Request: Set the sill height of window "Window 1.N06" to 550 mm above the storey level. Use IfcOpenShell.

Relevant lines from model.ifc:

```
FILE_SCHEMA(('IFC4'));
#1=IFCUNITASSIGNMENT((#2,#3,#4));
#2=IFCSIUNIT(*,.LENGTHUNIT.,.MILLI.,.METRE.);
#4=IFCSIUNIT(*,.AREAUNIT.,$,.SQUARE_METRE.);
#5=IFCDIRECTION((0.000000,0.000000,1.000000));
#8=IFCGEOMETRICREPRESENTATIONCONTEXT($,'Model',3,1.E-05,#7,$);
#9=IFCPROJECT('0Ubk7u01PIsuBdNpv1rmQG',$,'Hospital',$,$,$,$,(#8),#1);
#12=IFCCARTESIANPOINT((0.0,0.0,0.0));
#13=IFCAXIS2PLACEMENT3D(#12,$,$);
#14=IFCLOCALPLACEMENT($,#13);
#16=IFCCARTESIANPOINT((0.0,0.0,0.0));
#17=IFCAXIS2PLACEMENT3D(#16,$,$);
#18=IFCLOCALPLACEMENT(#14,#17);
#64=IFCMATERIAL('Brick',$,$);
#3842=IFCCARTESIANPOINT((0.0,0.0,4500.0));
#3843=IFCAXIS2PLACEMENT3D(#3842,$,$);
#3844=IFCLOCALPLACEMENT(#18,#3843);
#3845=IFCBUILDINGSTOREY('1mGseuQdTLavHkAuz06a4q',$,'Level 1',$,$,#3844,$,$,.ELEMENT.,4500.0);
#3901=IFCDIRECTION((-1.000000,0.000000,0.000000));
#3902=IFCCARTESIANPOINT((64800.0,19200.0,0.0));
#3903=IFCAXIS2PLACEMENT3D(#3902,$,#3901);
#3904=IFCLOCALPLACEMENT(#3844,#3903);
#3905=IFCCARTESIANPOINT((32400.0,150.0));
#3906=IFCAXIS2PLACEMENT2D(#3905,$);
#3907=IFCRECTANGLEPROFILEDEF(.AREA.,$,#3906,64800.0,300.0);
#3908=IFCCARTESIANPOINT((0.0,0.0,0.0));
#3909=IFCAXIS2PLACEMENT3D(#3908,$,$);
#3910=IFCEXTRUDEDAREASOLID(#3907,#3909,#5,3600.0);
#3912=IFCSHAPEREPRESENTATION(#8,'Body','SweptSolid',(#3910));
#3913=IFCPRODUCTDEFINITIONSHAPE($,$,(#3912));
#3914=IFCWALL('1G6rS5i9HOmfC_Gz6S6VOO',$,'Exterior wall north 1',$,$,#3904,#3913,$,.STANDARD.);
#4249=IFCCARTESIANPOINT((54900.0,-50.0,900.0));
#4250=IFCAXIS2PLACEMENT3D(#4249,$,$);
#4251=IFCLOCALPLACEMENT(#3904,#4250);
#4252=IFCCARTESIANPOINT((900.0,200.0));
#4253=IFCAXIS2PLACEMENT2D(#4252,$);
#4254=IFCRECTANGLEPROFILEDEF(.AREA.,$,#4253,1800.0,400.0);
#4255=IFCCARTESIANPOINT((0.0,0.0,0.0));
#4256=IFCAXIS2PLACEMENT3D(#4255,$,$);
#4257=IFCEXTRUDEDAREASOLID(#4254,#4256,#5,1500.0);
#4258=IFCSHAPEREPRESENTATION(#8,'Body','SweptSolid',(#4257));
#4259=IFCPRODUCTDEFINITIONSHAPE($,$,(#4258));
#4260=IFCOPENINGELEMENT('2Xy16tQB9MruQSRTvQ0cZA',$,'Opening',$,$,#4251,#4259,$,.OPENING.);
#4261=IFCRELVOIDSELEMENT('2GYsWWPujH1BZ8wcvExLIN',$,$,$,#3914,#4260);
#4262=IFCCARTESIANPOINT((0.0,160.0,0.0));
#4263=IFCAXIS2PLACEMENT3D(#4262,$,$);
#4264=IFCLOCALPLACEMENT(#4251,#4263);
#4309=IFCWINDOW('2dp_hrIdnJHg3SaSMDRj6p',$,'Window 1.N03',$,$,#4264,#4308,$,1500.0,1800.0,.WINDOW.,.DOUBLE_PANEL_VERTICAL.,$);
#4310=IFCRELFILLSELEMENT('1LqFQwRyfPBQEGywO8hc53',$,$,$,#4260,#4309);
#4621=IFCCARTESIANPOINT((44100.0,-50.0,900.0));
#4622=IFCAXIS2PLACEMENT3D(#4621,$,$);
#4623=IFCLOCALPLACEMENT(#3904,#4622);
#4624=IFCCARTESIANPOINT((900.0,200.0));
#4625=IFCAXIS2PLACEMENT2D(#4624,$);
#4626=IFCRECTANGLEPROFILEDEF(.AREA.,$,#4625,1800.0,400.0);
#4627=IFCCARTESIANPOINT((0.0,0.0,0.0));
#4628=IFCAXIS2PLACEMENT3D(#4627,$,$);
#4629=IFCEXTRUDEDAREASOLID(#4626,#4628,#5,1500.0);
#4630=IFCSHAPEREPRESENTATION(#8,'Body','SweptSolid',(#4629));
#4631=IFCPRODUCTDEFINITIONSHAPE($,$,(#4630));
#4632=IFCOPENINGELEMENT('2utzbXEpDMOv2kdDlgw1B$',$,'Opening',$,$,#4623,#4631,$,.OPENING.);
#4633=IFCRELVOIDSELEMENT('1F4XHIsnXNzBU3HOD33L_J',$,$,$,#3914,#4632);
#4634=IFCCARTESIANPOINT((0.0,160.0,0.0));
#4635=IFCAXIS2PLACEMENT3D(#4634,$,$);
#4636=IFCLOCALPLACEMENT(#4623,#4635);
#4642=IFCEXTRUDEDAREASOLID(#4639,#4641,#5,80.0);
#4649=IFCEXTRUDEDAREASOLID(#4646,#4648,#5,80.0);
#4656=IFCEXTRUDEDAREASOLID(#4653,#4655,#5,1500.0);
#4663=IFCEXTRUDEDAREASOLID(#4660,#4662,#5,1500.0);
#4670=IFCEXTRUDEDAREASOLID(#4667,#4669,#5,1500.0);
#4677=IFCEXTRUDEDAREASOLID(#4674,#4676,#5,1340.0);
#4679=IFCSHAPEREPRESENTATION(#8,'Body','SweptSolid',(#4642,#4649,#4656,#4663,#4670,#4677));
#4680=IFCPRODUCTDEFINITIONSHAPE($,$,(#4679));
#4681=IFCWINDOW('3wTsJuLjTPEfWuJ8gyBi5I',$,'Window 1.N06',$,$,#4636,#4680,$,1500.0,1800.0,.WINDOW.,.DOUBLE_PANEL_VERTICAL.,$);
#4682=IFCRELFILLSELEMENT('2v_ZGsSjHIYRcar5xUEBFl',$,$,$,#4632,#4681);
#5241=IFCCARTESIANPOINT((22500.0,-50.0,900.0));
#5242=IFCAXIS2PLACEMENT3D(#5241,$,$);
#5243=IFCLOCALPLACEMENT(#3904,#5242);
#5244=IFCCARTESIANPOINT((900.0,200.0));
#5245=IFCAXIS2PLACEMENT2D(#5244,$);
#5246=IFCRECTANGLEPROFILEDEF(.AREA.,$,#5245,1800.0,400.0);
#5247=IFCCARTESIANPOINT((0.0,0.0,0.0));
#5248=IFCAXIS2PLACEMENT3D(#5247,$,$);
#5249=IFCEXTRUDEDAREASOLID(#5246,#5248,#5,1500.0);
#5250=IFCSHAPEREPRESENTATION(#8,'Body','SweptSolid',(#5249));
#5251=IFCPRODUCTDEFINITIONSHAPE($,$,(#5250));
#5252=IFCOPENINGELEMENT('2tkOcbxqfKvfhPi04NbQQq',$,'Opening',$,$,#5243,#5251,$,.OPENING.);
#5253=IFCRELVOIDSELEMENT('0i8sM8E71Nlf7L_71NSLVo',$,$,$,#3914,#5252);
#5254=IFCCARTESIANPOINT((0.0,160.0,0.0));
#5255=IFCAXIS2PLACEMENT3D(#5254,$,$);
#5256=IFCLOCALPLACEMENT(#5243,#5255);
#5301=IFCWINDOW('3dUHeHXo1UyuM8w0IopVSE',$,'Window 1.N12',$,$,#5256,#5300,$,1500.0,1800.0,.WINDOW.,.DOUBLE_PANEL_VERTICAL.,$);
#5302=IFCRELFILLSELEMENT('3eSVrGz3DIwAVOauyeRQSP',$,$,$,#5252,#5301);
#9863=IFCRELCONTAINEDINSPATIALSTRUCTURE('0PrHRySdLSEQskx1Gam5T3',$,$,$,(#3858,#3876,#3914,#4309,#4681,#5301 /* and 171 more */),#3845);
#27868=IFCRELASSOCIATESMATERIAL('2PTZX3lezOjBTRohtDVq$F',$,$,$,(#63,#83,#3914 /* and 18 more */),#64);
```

```python
import numpy as np
import ifcopenshell
import ifcopenshell.api.geometry
import ifcopenshell.geom
import ifcopenshell.util.element
import ifcopenshell.util.placement
import ifcopenshell.util.shape
import ifcopenshell.util.unit

model = ifcopenshell.open("model.ifc")
unit_scale = ifcopenshell.util.unit.calculate_unit_scale(model)

window = model.by_guid("3wTsJuLjTPEfWuJ8gyBi5I")
opening = window.FillsVoids[0].RelatingOpeningElement
storey = ifcopenshell.util.element.get_container(window, ifc_class="IfcBuildingStorey")
level = ifcopenshell.util.placement.get_local_placement(storey.ObjectPlacement)[2, 3]

# The opening's origin need not be at the sill, so measure its lowest point.
shape = ifcopenshell.geom.create_shape(ifcopenshell.geom.settings(), opening)
bottom = ifcopenshell.util.shape.get_shape_bottom_elevation(shape, shape.geometry) / unit_scale
dz = level + 550.0 - bottom

shift = np.array([0.0, 0.0, dz])
# The window is placed relative to its opening, so it follows when the opening moves.
matrix = ifcopenshell.util.placement.get_local_placement(opening.ObjectPlacement)
matrix[:3, 3] += shift
ifcopenshell.api.geometry.edit_object_placement(
    model, product=opening, matrix=matrix, is_si=False, should_transform_children=True
)

print(f"moved by {dz * unit_scale:+.3f} m")

model.write("model-out.ifc")
```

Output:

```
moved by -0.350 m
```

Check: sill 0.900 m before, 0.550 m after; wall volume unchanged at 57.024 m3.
